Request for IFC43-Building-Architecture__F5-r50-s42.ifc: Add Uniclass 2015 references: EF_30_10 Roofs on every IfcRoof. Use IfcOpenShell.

First a look at what the model holds.

```python
import ifcopenshell

model = ifcopenshell.open("IFC43-Building-Architecture__F5-r50-s42.ifc")
print(model.schema)
print("classifications:", [c.Name for c in model.by_type("IfcClassification")])
for ifc_class in ("IfcDoor", "IfcRoof", "IfcStair", "IfcWall", "IfcWindow"):
    print(ifc_class, len(model.by_type(ifc_class)))
```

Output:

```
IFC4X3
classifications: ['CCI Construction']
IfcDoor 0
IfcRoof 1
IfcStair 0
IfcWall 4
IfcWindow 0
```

```python
import ifcopenshell
import ifcopenshell.api.classification

model = ifcopenshell.open("IFC43-Building-Architecture__F5-r50-s42.ifc")

system = ifcopenshell.api.classification.add_classification(model, classification="Uniclass 2015")

codes = {
    "IfcRoof": ("EF_30_10", "Roofs"),
}
for ifc_class, (code, name) in codes.items():
    products = model.by_type(ifc_class)
    ifcopenshell.api.classification.add_reference(
        model, products=products, classification=system, identification=code, name=name
    )
    print(code, len(products))

model.write("IFC43-Building-Architecture__F5-r50-s42_updated.ifc")
```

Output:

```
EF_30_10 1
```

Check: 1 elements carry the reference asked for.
